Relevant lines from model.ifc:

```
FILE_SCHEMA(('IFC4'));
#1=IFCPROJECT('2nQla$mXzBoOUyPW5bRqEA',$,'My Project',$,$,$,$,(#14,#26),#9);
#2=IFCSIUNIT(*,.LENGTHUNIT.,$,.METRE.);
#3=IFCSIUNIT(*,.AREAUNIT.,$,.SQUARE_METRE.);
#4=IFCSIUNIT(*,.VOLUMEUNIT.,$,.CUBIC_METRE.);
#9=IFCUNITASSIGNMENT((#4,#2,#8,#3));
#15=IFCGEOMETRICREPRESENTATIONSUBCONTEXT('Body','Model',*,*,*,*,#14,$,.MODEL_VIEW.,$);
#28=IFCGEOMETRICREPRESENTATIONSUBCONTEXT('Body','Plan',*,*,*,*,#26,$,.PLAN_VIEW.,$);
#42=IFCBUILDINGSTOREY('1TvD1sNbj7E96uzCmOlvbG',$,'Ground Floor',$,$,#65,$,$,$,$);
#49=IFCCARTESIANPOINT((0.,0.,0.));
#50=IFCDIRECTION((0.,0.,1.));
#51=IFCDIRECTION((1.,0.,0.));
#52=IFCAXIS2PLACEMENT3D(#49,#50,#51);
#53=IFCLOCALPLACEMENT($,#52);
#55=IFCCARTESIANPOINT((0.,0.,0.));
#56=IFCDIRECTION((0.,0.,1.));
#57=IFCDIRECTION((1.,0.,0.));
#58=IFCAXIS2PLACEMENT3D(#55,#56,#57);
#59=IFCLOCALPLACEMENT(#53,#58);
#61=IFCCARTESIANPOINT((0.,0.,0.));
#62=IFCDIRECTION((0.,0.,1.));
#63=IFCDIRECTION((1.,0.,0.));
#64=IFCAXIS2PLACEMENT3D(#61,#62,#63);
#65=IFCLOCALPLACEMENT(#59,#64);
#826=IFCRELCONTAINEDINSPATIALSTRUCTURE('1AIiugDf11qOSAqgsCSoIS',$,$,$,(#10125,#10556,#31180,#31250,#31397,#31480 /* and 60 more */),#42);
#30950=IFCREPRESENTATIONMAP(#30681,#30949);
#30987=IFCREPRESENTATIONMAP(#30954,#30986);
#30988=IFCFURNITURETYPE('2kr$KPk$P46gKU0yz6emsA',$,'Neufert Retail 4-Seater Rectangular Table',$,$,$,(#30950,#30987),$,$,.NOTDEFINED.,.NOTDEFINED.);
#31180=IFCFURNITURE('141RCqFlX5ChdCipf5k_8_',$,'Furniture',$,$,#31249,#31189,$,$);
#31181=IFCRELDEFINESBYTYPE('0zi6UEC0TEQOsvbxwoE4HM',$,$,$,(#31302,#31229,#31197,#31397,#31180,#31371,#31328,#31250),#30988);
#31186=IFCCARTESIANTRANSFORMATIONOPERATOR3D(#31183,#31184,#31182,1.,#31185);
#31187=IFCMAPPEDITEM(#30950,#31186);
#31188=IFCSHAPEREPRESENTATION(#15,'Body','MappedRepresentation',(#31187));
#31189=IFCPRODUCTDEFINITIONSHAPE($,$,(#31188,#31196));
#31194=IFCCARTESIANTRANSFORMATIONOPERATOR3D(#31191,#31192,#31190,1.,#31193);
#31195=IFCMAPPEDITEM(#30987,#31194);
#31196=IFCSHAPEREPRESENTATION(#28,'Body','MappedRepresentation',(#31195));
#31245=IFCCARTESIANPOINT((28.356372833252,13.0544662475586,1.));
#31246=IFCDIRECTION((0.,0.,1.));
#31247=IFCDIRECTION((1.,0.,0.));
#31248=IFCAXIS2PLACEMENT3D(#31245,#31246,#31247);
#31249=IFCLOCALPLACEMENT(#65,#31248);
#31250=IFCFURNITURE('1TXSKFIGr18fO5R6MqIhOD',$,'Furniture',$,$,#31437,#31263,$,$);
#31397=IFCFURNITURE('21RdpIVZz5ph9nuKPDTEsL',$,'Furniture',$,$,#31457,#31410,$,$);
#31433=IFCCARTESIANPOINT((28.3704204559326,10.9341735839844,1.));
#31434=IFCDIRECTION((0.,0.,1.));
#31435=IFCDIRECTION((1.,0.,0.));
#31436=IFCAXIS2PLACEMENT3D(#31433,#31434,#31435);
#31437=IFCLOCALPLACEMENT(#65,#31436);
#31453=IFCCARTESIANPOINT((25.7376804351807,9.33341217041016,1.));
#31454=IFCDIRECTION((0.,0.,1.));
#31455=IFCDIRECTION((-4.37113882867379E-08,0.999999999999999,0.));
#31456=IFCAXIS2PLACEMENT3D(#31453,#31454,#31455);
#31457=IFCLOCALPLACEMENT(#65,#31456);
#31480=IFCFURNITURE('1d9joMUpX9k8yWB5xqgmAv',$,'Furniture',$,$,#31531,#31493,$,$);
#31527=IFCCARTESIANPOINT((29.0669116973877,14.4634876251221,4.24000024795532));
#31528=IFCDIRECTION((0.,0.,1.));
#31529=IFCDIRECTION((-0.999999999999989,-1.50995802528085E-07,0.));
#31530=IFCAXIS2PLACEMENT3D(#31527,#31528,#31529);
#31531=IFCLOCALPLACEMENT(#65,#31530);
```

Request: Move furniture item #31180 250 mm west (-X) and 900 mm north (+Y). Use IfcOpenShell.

```python
import ifcopenshell
import ifcopenshell.api.geometry
import ifcopenshell.util.placement
import ifcopenshell.util.unit

model = ifcopenshell.open("model.ifc")
unit_scale = ifcopenshell.util.unit.calculate_unit_scale(model)

item = model.by_guid("141RCqFlX5ChdCipf5k_8_")
matrix = ifcopenshell.util.placement.get_local_placement(item.ObjectPlacement)
matrix[0, 3] -= 0.25 / unit_scale
matrix[1, 3] += 0.9 / unit_scale
ifcopenshell.api.geometry.edit_object_placement(model, product=item, matrix=matrix, is_si=False)

print(ifcopenshell.util.placement.get_local_placement(item.ObjectPlacement).round(3) + 0.0)

model.write("model_edited.ifc")
```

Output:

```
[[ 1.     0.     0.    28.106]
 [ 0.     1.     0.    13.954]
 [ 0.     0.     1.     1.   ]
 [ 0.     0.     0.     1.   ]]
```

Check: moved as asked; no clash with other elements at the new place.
